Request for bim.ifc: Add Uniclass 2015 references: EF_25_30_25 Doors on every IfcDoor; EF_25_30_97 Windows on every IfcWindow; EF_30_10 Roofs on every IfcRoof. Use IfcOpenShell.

First a look at what the model holds.

```python
import ifcopenshell

model = ifcopenshell.open("bim.ifc")
print(model.schema)
print("classifications:", [c.Name for c in model.by_type("IfcClassification")])
for ifc_class in ("IfcDoor", "IfcRoof", "IfcStair", "IfcWall", "IfcWindow"):
    print(ifc_class, len(model.by_type(ifc_class)))
```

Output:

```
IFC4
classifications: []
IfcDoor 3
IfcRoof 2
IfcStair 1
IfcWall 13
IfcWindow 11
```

```python
import ifcopenshell
import ifcopenshell.api.classification

model = ifcopenshell.open("bim.ifc")

system = ifcopenshell.api.classification.add_classification(model, classification="Uniclass 2015")

codes = {
    "IfcDoor": ("EF_25_30_25", "Doors"),
    "IfcWindow": ("EF_25_30_97", "Windows"),
    "IfcRoof": ("EF_30_10", "Roofs"),
}
for ifc_class, (code, name) in codes.items():
    products = model.by_type(ifc_class)
    ifcopenshell.api.classification.add_reference(
        model, products=products, classification=system, identification=code, name=name
    )
    print(code, len(products))

model.write("bim_v2.ifc")
```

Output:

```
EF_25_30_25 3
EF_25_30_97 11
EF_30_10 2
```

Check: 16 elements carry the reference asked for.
